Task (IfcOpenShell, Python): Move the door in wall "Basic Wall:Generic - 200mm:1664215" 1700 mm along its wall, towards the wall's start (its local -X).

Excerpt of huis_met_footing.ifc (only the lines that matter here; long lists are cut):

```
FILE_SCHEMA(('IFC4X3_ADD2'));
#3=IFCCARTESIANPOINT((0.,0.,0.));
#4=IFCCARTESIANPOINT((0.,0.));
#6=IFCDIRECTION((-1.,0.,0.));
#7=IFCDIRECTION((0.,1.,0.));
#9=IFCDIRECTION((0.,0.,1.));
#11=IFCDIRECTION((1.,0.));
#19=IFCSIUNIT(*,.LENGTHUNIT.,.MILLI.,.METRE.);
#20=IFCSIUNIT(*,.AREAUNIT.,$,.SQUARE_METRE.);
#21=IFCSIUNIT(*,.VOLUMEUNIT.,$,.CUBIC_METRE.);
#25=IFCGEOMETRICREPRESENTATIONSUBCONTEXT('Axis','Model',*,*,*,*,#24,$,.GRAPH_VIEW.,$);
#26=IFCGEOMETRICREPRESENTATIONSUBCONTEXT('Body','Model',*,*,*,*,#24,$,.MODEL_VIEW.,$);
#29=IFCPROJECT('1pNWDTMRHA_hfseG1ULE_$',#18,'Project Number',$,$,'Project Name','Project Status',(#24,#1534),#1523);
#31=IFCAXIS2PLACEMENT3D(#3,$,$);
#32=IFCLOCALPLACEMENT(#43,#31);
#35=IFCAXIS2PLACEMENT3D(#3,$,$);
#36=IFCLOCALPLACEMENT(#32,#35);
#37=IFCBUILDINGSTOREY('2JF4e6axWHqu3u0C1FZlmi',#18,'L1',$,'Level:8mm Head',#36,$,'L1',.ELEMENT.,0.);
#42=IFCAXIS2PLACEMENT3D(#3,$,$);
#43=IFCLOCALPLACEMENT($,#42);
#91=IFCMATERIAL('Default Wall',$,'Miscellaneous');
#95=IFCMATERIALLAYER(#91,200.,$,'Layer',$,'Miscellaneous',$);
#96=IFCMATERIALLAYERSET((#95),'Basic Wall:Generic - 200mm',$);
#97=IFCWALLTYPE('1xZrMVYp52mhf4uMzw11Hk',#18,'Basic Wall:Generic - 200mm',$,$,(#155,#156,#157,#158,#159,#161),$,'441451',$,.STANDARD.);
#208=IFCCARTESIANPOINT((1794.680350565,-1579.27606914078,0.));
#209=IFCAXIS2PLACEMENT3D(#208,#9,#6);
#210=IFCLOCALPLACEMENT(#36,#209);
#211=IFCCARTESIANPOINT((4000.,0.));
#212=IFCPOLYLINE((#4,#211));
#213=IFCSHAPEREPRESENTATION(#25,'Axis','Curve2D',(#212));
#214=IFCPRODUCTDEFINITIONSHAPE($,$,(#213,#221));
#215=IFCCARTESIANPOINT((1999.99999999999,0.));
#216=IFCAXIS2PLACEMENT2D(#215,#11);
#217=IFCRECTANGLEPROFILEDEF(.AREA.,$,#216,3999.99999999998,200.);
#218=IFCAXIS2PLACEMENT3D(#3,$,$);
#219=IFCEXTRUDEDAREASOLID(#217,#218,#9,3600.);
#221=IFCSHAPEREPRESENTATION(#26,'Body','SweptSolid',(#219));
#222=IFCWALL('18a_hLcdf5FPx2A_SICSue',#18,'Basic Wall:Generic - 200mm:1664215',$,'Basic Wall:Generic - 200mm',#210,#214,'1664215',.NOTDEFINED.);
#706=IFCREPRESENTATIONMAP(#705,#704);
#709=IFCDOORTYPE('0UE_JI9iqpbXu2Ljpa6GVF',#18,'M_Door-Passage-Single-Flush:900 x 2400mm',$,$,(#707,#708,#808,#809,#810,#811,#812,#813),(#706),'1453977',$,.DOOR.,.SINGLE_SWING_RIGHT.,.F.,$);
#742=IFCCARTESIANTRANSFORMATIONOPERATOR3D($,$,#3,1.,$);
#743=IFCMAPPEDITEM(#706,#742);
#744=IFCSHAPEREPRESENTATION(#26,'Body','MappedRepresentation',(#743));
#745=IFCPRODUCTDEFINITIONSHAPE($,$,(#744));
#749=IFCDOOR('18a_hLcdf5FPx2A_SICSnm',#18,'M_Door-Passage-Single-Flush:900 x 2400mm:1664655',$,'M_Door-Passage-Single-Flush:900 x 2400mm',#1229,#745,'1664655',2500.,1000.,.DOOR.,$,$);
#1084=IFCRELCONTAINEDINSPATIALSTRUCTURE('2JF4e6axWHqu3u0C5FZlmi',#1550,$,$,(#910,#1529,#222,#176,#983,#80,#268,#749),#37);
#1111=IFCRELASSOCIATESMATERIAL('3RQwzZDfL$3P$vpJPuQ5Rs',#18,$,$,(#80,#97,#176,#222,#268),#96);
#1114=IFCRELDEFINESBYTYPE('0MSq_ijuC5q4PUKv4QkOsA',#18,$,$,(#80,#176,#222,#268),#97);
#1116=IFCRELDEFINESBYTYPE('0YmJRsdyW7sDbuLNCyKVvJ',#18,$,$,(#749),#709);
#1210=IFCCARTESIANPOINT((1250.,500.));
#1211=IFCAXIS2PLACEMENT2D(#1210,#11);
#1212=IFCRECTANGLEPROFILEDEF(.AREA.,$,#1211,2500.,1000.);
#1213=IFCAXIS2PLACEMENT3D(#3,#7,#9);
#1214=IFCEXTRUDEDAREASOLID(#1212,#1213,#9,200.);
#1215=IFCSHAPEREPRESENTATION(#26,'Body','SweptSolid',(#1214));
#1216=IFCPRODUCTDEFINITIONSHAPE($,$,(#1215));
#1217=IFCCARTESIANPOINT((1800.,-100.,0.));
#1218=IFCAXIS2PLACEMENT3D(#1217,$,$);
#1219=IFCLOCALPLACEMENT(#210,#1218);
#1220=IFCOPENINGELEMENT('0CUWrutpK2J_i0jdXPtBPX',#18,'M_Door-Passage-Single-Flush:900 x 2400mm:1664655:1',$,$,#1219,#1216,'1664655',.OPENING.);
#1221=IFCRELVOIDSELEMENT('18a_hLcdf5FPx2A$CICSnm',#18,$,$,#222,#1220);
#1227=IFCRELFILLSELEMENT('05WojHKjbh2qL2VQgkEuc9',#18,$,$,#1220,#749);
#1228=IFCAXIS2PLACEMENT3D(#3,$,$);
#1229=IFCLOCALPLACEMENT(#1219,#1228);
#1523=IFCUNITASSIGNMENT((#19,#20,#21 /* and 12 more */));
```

```python
import ifcopenshell
import ifcopenshell.api.geometry
import ifcopenshell.util.placement
import ifcopenshell.util.unit

model = ifcopenshell.open("huis_met_footing.ifc")
unit_scale = ifcopenshell.util.unit.calculate_unit_scale(model)

door = model.by_guid("18a_hLcdf5FPx2A_SICSnm")
opening = door.FillsVoids[0].RelatingOpeningElement
wall = opening.VoidsElements[0].RelatingBuildingElement

wall_matrix = ifcopenshell.util.placement.get_local_placement(wall.ObjectPlacement)
shift = wall_matrix[:3, 0] * -1.7 / unit_scale
before = ifcopenshell.util.placement.get_local_placement(door.ObjectPlacement)[:3, 3].copy()

# The door is placed relative to its opening, so it follows when the opening moves.
matrix = ifcopenshell.util.placement.get_local_placement(opening.ObjectPlacement)
matrix[:3, 3] += shift
ifcopenshell.api.geometry.edit_object_placement(
    model, product=opening, matrix=matrix, is_si=False, should_transform_children=True
)

after = ifcopenshell.util.placement.get_local_placement(door.ObjectPlacement)[:3, 3]
print("door moved by", (after - before).round(3) + 0.0)

model.write("huis_met_footing_edited.ifc")
```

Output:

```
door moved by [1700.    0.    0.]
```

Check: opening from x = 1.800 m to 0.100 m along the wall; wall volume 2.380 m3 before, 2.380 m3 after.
